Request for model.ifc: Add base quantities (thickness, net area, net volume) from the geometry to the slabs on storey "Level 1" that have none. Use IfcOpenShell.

First a look at what the model holds.

```python
import ifcopenshell
import ifcopenshell.util.element
import ifcopenshell.util.unit

model = ifcopenshell.open("model.ifc")
print(model.schema)
for unit_type in ("LENGTHUNIT", "AREAUNIT", "VOLUMEUNIT"):
    print(unit_type, ifcopenshell.util.unit.calculate_unit_scale(model, unit_type))
storey = next(s for s in model.by_type("IfcBuildingStorey") if s.Name == "Level 1")
slabs = [e for e in ifcopenshell.util.element.get_decomposition(storey) if e.is_a("IfcSlab")]
for e in sorted(slabs, key=lambda e: e.id()):
    print(e.id(), e.is_a(), e.Name, list(ifcopenshell.util.element.get_psets(e, qtos_only=True)), sep=" | ")
```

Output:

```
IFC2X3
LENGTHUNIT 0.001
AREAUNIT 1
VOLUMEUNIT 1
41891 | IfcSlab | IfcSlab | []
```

```python
import ifcopenshell
import ifcopenshell.api.pset
import ifcopenshell.geom
import ifcopenshell.util.element
import ifcopenshell.util.shape
import ifcopenshell.util.unit

model = ifcopenshell.open("model.ifc")
unit_scale = ifcopenshell.util.unit.calculate_unit_scale(model)
area_scale = ifcopenshell.util.unit.calculate_unit_scale(model, "AREAUNIT")
volume_scale = ifcopenshell.util.unit.calculate_unit_scale(model, "VOLUMEUNIT")
settings = ifcopenshell.geom.settings()

storey = next(s for s in model.by_type("IfcBuildingStorey") if s.Name == "Level 1")
slabs = [e for e in ifcopenshell.util.element.get_decomposition(storey) if e.is_a("IfcSlab")]

for e in sorted(slabs, key=lambda e: e.id()):
    if ifcopenshell.util.element.get_psets(e, qtos_only=True, should_inherit=False):
        continue
    # Geometry comes back in metres, in the element's own axes.
    shape = ifcopenshell.geom.create_shape(settings, e)
    values = {
        "Width": ifcopenshell.util.shape.get_z(shape.geometry) / unit_scale,
        "NetArea": ifcopenshell.util.shape.get_footprint_area(shape.geometry) / area_scale,
        "NetVolume": ifcopenshell.util.shape.get_volume(shape.geometry) / volume_scale,
    }
    qto = ifcopenshell.api.pset.add_qto(model, product=e, name="BaseQuantities")
    ifcopenshell.api.pset.edit_qto(model, qto=qto, properties=values)
    print(e.id(), {k: round(v, 3) for k, v in values.items()})

model.write("model-out.ifc")
```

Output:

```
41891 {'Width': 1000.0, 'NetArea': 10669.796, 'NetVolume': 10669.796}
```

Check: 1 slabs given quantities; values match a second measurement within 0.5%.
